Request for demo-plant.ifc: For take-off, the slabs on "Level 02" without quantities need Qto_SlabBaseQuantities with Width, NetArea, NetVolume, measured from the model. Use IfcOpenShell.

First a look at what the model holds.

```python
import ifcopenshell
import ifcopenshell.util.element
import ifcopenshell.util.unit

model = ifcopenshell.open("demo-plant.ifc")
print(model.schema)
for unit_type in ("LENGTHUNIT", "AREAUNIT", "VOLUMEUNIT"):
    print(unit_type, ifcopenshell.util.unit.calculate_unit_scale(model, unit_type))
storey = next(s for s in model.by_type("IfcBuildingStorey") if s.Name == "Level 02")
slabs = [e for e in ifcopenshell.util.element.get_decomposition(storey) if e.is_a("IfcSlab")]
for e in sorted(slabs, key=lambda e: e.id()):
    print(e.id(), e.is_a(), e.Name, list(ifcopenshell.util.element.get_psets(e, qtos_only=True)), sep=" | ")
```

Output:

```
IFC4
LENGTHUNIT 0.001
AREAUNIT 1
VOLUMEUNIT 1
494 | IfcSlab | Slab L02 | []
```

```python
import ifcopenshell
import ifcopenshell.api.pset
import ifcopenshell.geom
import ifcopenshell.util.element
import ifcopenshell.util.shape
import ifcopenshell.util.unit

model = ifcopenshell.open("demo-plant.ifc")
unit_scale = ifcopenshell.util.unit.calculate_unit_scale(model)
area_scale = ifcopenshell.util.unit.calculate_unit_scale(model, "AREAUNIT")
volume_scale = ifcopenshell.util.unit.calculate_unit_scale(model, "VOLUMEUNIT")
settings = ifcopenshell.geom.settings()

storey = next(s for s in model.by_type("IfcBuildingStorey") if s.Name == "Level 02")
slabs = [e for e in ifcopenshell.util.element.get_decomposition(storey) if e.is_a("IfcSlab")]

for e in sorted(slabs, key=lambda e: e.id()):
    if ifcopenshell.util.element.get_psets(e, qtos_only=True, should_inherit=False):
        continue
    # Geometry comes back in metres, in the element's own axes.
    shape = ifcopenshell.geom.create_shape(settings, e)
    values = {
        "Width": ifcopenshell.util.shape.get_z(shape.geometry) / unit_scale,
        "NetArea": ifcopenshell.util.shape.get_footprint_area(shape.geometry) / area_scale,
        "NetVolume": ifcopenshell.util.shape.get_volume(shape.geometry) / volume_scale,
    }
    qto = ifcopenshell.api.pset.add_qto(model, product=e, name="Qto_SlabBaseQuantities")
    ifcopenshell.api.pset.edit_qto(model, qto=qto, properties=values)
    print(e.id(), {k: round(v, 3) for k, v in values.items()})

model.write("demo-plant_rev.ifc")
```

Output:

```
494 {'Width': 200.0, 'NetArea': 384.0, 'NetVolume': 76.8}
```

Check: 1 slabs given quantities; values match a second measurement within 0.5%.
